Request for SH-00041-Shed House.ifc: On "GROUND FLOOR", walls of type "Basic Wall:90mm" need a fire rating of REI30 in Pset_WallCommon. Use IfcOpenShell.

First a look at what the model holds.

```python
import ifcopenshell
import ifcopenshell.util.element

model = ifcopenshell.open("SH-00041-Shed House.ifc")
print(model.schema)
storey = next(s for s in model.by_type("IfcBuildingStorey") if s.Name == "GROUND FLOOR")
walls = [e for e in ifcopenshell.util.element.get_decomposition(storey) if e.is_a("IfcWall")]
seen = {}
for e in walls:
    element_type = ifcopenshell.util.element.get_type(e)
    key = (element_type.Name if element_type != e and element_type else None, ifcopenshell.util.element.get_pset(e, "Pset_WallCommon", "FireRating"))
    seen[key] = seen.get(key, 0) + 1
for (name, value), count in sorted(seen.items(), key=str):
    print(count, "x", name, "|", value)
```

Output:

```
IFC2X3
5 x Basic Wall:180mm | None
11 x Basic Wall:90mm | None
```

```python
import ifcopenshell
import ifcopenshell.api.pset
import ifcopenshell.util.element

model = ifcopenshell.open("SH-00041-Shed House.ifc")

storey = next(s for s in model.by_type("IfcBuildingStorey") if s.Name == "GROUND FLOOR")
walls = [e for e in ifcopenshell.util.element.get_decomposition(storey) if e.is_a("IfcWall")]

count = 0
for e in walls:
    element_type = ifcopenshell.util.element.get_type(e)
    if element_type in (None, e) or element_type.Name != "Basic Wall:90mm":
        continue
    # add_pset returns the element's existing set when there is one.
    pset = ifcopenshell.api.pset.add_pset(model, product=e, name="Pset_WallCommon")
    ifcopenshell.api.pset.edit_pset(model, pset=pset, properties={"FireRating": "REI30"})
    count += 1

print(count, "walls updated")

model.write("SH-00041-Shed House_updated.ifc")
```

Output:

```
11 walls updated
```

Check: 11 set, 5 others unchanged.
